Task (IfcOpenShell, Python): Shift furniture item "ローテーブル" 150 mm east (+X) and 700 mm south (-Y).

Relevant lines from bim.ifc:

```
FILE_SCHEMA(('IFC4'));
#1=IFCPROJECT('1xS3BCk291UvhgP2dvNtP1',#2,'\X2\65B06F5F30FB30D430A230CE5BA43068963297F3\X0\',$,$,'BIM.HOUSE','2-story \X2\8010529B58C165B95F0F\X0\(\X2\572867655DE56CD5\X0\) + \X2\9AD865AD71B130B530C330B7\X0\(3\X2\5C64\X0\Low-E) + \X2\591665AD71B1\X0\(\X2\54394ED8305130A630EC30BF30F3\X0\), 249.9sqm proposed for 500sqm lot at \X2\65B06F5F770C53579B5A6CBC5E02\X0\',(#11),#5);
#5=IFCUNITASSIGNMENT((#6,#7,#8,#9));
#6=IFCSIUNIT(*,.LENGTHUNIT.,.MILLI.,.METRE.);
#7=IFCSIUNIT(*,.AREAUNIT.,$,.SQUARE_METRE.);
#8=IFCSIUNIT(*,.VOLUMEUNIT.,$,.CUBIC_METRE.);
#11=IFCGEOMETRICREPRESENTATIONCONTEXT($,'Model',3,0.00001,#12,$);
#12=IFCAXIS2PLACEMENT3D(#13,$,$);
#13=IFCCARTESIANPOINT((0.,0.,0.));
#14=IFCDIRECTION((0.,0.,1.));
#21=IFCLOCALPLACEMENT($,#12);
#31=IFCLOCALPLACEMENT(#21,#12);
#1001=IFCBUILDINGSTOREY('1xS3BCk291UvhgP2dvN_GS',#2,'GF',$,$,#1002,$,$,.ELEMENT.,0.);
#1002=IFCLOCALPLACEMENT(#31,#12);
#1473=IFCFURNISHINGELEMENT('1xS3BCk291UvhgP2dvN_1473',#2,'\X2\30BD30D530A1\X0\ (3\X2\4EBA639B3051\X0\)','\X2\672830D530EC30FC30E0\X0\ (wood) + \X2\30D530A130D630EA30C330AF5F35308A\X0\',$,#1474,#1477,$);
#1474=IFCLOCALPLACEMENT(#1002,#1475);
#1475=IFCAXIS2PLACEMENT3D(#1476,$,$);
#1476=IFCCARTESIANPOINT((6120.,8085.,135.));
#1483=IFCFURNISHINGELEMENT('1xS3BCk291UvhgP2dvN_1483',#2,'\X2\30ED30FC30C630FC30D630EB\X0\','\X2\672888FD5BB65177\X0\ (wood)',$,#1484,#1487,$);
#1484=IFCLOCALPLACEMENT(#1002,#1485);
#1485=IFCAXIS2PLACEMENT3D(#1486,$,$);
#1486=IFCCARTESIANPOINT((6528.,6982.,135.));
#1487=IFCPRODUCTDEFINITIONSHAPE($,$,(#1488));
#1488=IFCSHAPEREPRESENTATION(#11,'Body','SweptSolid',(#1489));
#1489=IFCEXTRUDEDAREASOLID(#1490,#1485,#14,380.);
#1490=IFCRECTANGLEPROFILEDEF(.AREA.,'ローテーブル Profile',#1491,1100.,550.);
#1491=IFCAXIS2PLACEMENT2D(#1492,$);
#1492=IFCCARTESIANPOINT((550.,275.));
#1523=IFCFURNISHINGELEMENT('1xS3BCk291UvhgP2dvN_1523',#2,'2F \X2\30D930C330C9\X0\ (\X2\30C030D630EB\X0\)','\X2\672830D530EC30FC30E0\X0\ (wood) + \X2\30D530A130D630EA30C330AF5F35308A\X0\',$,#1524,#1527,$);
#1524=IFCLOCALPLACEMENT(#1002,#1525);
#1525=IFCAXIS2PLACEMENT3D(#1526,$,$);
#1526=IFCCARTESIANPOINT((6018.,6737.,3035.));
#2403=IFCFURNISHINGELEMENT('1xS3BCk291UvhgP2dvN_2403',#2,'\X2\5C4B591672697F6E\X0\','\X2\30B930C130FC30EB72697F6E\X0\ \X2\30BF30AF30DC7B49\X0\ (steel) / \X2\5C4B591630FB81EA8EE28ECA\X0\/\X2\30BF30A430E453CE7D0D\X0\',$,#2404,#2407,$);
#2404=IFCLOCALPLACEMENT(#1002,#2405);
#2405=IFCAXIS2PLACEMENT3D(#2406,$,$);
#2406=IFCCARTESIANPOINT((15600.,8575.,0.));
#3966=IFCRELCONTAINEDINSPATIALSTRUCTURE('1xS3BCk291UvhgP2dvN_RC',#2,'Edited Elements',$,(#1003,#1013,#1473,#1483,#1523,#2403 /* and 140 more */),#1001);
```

```python
import ifcopenshell
import ifcopenshell.api.geometry
import ifcopenshell.util.placement

model = ifcopenshell.open("bim.ifc")

item = model.by_id(1483)
matrix = ifcopenshell.util.placement.get_local_placement(item.ObjectPlacement)
matrix[0, 3] += 150.0
matrix[1, 3] -= 700.0
ifcopenshell.api.geometry.edit_object_placement(model, product=item, matrix=matrix, is_si=False)

print(ifcopenshell.util.placement.get_local_placement(item.ObjectPlacement).round(3) + 0.0)

model.write("bim_updated.ifc")
```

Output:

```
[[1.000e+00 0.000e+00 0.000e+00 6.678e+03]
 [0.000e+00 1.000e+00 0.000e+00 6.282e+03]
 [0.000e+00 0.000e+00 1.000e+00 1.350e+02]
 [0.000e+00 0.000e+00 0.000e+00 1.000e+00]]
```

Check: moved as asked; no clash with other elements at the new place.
